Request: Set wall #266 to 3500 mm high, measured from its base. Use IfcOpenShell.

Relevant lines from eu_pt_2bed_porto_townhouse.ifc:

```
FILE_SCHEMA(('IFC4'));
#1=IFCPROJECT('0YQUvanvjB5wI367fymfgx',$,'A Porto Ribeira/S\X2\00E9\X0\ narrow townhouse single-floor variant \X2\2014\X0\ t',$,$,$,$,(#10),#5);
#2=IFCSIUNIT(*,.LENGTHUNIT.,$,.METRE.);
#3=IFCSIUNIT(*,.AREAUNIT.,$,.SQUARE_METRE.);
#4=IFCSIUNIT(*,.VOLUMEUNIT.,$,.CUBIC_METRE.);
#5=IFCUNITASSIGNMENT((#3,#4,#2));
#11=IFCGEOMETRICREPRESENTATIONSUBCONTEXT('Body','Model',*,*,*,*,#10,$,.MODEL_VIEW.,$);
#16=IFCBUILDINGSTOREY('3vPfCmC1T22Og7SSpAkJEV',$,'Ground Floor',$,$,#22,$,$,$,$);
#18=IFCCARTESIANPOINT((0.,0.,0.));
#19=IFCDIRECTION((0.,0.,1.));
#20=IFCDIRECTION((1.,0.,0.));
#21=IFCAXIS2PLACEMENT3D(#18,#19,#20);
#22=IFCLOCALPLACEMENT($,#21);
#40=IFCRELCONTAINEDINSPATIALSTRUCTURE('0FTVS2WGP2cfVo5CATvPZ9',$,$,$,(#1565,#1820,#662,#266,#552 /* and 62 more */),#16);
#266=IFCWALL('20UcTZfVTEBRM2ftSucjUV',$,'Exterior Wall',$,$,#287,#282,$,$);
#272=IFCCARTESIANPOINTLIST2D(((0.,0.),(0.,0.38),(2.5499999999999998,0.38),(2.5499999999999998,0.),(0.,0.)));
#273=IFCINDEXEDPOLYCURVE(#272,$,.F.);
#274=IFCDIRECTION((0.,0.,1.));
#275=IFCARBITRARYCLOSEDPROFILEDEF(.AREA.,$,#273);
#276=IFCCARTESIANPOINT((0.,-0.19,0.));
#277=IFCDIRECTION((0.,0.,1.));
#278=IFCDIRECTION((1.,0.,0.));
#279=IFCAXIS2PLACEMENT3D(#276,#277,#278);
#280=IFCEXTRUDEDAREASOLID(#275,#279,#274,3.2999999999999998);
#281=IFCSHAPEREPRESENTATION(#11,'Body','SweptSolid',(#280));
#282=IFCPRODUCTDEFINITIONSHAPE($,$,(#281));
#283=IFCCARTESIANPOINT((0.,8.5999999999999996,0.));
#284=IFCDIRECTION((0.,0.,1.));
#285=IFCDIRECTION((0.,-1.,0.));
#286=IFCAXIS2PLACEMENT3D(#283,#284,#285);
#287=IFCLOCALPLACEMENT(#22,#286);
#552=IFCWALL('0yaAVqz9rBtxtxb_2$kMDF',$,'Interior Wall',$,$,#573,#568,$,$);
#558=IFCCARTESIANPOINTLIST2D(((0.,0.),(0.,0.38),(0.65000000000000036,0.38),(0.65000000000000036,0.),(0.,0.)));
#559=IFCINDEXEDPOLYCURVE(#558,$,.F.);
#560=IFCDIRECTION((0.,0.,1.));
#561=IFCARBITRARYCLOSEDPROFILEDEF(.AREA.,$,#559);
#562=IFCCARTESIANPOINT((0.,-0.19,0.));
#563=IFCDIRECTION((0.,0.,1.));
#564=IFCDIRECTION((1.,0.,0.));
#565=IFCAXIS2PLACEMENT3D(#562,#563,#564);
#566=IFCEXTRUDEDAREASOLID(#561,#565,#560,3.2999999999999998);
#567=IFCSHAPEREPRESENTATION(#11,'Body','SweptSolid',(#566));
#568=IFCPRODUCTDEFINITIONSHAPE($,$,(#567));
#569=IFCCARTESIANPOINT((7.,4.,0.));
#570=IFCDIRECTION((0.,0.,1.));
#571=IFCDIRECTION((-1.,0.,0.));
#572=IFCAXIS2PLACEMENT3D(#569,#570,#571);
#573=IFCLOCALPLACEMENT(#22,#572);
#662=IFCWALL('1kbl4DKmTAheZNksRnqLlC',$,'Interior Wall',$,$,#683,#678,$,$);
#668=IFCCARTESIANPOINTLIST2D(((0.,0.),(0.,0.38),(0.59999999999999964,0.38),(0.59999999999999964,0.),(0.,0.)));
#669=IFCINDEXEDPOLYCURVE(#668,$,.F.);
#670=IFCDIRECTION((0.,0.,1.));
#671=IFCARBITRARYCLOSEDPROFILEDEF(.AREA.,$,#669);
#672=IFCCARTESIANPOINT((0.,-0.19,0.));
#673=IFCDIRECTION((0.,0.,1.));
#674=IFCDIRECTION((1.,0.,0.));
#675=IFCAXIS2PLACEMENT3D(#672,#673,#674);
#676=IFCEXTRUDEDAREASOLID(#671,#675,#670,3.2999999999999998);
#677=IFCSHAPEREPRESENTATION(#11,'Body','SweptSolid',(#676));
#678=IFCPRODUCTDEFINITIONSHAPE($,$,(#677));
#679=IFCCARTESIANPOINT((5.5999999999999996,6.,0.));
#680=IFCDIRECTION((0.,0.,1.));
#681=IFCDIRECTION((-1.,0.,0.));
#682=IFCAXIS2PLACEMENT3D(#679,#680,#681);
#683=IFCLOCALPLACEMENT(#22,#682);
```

```python
import ifcopenshell
import ifcopenshell.geom
import ifcopenshell.util.representation
import ifcopenshell.util.shape
import ifcopenshell.util.unit

model = ifcopenshell.open("eu_pt_2bed_porto_townhouse.ifc")
unit_scale = ifcopenshell.util.unit.calculate_unit_scale(model)
settings = ifcopenshell.geom.settings()


def volume(element):
    """Net volume in cubic metres, openings subtracted."""
    shape = ifcopenshell.geom.create_shape(settings, element)
    return ifcopenshell.util.shape.get_volume(shape.geometry)


wall = model.by_id(266)
before = volume(wall)

body = ifcopenshell.util.representation.get_representation(wall, "Model", "Body")
solid = body.Items[0]
old_height = solid.Depth
solid.Depth = 3.5 / unit_scale
after = volume(wall)

print(f"height {old_height:g} -> {solid.Depth:g}, volume {before:.3f} -> {after:.3f} m3")

model.write("eu_pt_2bed_porto_townhouse_updated.ifc")
```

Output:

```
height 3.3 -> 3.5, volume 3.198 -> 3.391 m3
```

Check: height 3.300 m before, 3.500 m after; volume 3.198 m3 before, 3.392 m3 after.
